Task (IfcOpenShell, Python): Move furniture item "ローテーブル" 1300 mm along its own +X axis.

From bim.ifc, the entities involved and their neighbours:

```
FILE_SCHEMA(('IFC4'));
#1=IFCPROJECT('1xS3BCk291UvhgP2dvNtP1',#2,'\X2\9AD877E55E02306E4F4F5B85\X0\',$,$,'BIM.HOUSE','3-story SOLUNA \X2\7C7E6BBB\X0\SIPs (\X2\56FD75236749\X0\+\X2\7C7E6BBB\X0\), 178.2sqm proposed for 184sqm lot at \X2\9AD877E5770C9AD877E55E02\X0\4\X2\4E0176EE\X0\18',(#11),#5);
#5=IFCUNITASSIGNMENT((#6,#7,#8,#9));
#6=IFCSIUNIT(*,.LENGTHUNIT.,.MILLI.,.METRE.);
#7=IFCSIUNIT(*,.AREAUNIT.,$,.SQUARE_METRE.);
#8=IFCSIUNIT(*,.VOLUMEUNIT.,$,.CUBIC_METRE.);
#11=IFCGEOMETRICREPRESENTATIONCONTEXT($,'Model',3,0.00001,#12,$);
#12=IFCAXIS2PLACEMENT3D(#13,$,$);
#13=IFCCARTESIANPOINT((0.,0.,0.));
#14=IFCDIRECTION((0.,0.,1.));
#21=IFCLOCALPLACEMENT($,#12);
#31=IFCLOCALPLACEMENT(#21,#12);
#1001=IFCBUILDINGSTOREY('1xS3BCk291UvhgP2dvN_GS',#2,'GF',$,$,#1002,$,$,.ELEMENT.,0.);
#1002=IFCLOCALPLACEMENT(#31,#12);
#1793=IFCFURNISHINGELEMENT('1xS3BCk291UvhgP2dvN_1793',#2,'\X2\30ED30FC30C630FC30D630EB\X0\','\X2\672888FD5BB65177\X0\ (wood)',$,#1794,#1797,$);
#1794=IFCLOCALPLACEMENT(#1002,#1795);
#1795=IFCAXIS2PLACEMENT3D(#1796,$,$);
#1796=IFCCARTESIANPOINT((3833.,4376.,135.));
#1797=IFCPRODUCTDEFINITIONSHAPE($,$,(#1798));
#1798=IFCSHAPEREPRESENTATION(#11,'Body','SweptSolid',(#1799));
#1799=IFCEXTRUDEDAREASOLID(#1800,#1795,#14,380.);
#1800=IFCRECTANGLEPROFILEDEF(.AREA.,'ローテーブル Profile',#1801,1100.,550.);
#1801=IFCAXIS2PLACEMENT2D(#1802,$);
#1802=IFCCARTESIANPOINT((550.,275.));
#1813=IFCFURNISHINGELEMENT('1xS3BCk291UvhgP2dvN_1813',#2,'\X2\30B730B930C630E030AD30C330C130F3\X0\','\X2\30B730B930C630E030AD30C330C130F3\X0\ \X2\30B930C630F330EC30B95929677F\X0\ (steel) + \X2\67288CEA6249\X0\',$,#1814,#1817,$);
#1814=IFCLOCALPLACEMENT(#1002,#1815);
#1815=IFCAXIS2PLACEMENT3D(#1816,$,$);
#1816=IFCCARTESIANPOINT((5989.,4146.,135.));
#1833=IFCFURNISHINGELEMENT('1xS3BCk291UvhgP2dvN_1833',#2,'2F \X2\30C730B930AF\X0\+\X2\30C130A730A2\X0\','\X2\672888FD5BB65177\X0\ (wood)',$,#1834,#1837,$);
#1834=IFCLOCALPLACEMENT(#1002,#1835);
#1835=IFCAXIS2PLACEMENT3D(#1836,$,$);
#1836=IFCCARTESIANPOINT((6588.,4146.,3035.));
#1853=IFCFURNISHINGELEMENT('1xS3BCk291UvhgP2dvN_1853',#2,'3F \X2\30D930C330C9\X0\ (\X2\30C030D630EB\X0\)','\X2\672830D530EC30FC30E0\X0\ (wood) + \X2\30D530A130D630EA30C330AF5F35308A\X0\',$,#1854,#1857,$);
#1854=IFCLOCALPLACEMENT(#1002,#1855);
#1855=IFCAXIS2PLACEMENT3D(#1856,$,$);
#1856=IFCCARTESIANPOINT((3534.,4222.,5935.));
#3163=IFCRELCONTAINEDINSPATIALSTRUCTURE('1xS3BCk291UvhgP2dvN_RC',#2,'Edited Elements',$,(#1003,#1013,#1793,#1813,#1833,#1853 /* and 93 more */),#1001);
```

```python
import ifcopenshell
import ifcopenshell.api.geometry
import ifcopenshell.util.placement
import ifcopenshell.util.unit

model = ifcopenshell.open("bim.ifc")
unit_scale = ifcopenshell.util.unit.calculate_unit_scale(model)

item = model.by_guid("1xS3BCk291UvhgP2dvN_1793")
matrix = ifcopenshell.util.placement.get_local_placement(item.ObjectPlacement)
matrix[:3, 3] += matrix[:3, 0] * 1.3 / unit_scale
ifcopenshell.api.geometry.edit_object_placement(model, product=item, matrix=matrix, is_si=False)

print(ifcopenshell.util.placement.get_local_placement(item.ObjectPlacement).round(3) + 0.0)

model.write("bim-out.ifc")
```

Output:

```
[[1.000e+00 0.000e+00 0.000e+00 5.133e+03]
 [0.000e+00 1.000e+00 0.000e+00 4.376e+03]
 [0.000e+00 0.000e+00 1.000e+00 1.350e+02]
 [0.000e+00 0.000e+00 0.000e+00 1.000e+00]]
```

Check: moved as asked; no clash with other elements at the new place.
